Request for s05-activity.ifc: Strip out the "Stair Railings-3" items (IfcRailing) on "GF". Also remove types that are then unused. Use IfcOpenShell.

First a look at what the model holds.

```python
import ifcopenshell
import ifcopenshell.util.element

model = ifcopenshell.open("s05-activity.ifc")
print(model.schema)
storey = next(s for s in model.by_type("IfcBuildingStorey") if s.Name == "GF")
railings = [e for e in ifcopenshell.util.element.get_decomposition(storey) if e.is_a("IfcRailing")]
seen = {}
for e in railings:
    element_type = ifcopenshell.util.element.get_type(e)
    name = element_type.Name if element_type not in (None, e) else None
    seen[name] = seen.get(name, 0) + 1
for name, count in sorted(seen.items(), key=str):
    print(count, "x", name)
```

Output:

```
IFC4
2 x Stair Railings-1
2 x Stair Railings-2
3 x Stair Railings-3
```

```python
import ifcopenshell
import ifcopenshell.api.root
import ifcopenshell.util.element

model = ifcopenshell.open("s05-activity.ifc")

storey = next(s for s in model.by_type("IfcBuildingStorey") if s.Name == "GF")
railings = [e for e in ifcopenshell.util.element.get_decomposition(storey) if e.is_a("IfcRailing")]
targets = [e for e in railings if (t := ifcopenshell.util.element.get_type(e)) not in (None, e) and t.Name == "Stair Railings-3"]
types = {ifcopenshell.util.element.get_type(e) for e in targets} - {None, *targets}

for e in targets:
    ifcopenshell.api.root.remove_product(model, product=e)
print(len(targets), "removed")

unused = [t for t in types if not ifcopenshell.util.element.get_types(t)]
for t in unused:
    ifcopenshell.api.root.remove_product(model, product=t)
print(len(unused), "unused types removed")

model.write("s05-activity_edited.ifc")
```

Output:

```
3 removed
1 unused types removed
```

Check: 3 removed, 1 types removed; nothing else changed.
